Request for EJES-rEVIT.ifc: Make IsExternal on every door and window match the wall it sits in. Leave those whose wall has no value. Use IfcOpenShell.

First a look at what the model holds.

```python
import ifcopenshell
import ifcopenshell.util.element

model = ifcopenshell.open("EJES-rEVIT.ifc")
print(model.schema)
seen = {}
for e in model.by_type("IfcDoor") + model.by_type("IfcWindow"):
    if not e.FillsVoids:
        continue
    host = e.FillsVoids[0].RelatingOpeningElement.VoidsElements[0].RelatingBuildingElement
    own = ifcopenshell.util.element.get_pset(e, f"Pset_{e.is_a()[3:].removesuffix('StandardCase')}Common", "IsExternal")
    wall = ifcopenshell.util.element.get_pset(host, "Pset_WallCommon", "IsExternal")
    seen[e.is_a(), own, wall] = seen.get((e.is_a(), own, wall), 0) + 1
for (cls, own, wall), count in sorted(seen.items(), key=str):
    print(count, cls, "IsExternal:", own, "| host wall:", wall)
```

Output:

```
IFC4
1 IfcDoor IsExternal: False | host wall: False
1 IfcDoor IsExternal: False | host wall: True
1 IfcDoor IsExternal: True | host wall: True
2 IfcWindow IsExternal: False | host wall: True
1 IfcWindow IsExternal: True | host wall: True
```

```python
import ifcopenshell
import ifcopenshell.api.pset
import ifcopenshell.util.element

model = ifcopenshell.open("EJES-rEVIT.ifc")

count = 0
for ifc_class, pset_name in (("IfcDoor", "Pset_DoorCommon"), ("IfcWindow", "Pset_WindowCommon")):
    for e in model.by_type(ifc_class):
        if not e.FillsVoids:
            continue
        host = e.FillsVoids[0].RelatingOpeningElement.VoidsElements[0].RelatingBuildingElement
        external = ifcopenshell.util.element.get_pset(host, "Pset_WallCommon", "IsExternal")
        if external is None or ifcopenshell.util.element.get_pset(e, pset_name, "IsExternal") == external:
            continue
        pset = ifcopenshell.api.pset.add_pset(model, product=e, name=pset_name)
        ifcopenshell.api.pset.edit_pset(model, pset=pset, properties={"IsExternal": external})
        count += 1

print(count, "updated")

model.write("EJES-rEVIT-out.ifc")
```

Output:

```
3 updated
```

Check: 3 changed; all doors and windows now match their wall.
